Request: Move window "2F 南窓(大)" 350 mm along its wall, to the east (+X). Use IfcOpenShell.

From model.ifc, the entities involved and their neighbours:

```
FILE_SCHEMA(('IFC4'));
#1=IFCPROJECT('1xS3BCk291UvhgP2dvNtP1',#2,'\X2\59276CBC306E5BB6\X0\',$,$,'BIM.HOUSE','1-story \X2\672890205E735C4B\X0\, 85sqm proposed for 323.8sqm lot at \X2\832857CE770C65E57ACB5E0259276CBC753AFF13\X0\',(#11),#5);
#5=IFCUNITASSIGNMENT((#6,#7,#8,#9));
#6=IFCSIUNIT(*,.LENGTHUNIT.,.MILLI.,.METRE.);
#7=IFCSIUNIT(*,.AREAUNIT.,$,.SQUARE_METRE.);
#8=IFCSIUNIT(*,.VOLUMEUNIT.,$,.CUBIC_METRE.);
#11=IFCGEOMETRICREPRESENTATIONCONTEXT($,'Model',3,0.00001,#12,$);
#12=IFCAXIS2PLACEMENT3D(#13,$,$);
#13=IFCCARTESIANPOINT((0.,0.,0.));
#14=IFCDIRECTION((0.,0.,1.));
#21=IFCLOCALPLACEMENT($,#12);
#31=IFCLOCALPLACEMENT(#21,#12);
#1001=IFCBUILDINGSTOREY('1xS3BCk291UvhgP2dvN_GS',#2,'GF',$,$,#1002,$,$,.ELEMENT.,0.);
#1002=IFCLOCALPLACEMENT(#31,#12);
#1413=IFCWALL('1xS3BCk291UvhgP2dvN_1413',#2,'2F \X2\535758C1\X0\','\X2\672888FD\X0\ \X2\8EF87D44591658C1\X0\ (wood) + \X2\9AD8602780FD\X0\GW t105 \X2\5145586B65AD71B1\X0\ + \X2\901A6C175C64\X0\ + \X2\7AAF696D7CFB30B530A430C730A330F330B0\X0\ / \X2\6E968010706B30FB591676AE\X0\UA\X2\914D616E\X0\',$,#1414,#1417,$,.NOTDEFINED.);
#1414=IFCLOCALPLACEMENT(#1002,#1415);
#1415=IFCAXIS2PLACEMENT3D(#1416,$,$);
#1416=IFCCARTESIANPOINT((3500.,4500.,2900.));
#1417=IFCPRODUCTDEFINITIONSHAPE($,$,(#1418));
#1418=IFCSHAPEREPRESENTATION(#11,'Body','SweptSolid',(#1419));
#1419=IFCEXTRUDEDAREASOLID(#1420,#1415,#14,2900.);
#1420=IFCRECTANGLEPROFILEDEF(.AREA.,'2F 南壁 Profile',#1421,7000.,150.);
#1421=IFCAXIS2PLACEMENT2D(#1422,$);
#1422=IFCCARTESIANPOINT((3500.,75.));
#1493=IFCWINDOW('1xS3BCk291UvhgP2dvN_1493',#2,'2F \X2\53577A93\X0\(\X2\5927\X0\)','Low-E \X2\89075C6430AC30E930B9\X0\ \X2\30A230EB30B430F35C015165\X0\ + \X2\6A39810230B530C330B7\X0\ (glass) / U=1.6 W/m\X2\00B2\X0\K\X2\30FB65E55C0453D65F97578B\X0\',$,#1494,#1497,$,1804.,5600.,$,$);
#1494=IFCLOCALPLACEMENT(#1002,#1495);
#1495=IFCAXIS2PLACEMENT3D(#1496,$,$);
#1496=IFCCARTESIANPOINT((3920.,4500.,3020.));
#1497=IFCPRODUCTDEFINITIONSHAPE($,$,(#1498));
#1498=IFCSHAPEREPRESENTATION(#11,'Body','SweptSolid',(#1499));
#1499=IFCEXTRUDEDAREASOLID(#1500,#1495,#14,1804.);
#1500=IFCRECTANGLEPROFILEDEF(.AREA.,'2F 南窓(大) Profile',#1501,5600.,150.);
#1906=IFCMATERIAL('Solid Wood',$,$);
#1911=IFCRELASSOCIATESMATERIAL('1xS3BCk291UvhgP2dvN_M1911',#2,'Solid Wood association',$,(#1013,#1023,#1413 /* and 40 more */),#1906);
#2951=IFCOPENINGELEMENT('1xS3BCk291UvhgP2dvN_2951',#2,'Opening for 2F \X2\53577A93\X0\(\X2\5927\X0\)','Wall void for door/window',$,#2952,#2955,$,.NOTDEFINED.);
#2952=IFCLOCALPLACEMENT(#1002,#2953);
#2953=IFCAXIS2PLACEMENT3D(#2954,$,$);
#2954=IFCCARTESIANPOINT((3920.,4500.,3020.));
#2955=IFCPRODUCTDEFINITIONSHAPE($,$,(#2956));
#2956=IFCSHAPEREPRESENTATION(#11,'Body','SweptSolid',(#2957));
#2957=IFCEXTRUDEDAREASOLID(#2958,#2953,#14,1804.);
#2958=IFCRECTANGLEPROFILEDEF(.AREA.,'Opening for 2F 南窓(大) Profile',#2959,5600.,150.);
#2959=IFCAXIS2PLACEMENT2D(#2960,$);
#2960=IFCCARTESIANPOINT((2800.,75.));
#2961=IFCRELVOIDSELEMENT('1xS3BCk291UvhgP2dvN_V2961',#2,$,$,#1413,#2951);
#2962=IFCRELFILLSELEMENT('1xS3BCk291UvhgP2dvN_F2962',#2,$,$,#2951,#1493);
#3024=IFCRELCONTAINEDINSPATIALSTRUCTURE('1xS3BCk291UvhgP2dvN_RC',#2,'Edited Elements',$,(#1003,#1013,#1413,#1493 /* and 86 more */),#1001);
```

```python
import ifcopenshell
import ifcopenshell.api.geometry
import ifcopenshell.util.placement

model = ifcopenshell.open("model.ifc")

window = model.by_guid("1xS3BCk291UvhgP2dvN_1493")
opening = window.FillsVoids[0].RelatingOpeningElement
wall = opening.VoidsElements[0].RelatingBuildingElement

wall_matrix = ifcopenshell.util.placement.get_local_placement(wall.ObjectPlacement)
shift = wall_matrix[:3, 0] * 350.0
before = ifcopenshell.util.placement.get_local_placement(window.ObjectPlacement)[:3, 3].copy()

# The window is not placed relative to its opening, so move both.
for product in (opening, window):
    matrix = ifcopenshell.util.placement.get_local_placement(product.ObjectPlacement)
    matrix[:3, 3] += shift
    ifcopenshell.api.geometry.edit_object_placement(model, product=product, matrix=matrix, is_si=False)

after = ifcopenshell.util.placement.get_local_placement(window.ObjectPlacement)[:3, 3]
print("window moved by", (after - before).round(3) + 0.0)

model.write("model_v2.ifc")
```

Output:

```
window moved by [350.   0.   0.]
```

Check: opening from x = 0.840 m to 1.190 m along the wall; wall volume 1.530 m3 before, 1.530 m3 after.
